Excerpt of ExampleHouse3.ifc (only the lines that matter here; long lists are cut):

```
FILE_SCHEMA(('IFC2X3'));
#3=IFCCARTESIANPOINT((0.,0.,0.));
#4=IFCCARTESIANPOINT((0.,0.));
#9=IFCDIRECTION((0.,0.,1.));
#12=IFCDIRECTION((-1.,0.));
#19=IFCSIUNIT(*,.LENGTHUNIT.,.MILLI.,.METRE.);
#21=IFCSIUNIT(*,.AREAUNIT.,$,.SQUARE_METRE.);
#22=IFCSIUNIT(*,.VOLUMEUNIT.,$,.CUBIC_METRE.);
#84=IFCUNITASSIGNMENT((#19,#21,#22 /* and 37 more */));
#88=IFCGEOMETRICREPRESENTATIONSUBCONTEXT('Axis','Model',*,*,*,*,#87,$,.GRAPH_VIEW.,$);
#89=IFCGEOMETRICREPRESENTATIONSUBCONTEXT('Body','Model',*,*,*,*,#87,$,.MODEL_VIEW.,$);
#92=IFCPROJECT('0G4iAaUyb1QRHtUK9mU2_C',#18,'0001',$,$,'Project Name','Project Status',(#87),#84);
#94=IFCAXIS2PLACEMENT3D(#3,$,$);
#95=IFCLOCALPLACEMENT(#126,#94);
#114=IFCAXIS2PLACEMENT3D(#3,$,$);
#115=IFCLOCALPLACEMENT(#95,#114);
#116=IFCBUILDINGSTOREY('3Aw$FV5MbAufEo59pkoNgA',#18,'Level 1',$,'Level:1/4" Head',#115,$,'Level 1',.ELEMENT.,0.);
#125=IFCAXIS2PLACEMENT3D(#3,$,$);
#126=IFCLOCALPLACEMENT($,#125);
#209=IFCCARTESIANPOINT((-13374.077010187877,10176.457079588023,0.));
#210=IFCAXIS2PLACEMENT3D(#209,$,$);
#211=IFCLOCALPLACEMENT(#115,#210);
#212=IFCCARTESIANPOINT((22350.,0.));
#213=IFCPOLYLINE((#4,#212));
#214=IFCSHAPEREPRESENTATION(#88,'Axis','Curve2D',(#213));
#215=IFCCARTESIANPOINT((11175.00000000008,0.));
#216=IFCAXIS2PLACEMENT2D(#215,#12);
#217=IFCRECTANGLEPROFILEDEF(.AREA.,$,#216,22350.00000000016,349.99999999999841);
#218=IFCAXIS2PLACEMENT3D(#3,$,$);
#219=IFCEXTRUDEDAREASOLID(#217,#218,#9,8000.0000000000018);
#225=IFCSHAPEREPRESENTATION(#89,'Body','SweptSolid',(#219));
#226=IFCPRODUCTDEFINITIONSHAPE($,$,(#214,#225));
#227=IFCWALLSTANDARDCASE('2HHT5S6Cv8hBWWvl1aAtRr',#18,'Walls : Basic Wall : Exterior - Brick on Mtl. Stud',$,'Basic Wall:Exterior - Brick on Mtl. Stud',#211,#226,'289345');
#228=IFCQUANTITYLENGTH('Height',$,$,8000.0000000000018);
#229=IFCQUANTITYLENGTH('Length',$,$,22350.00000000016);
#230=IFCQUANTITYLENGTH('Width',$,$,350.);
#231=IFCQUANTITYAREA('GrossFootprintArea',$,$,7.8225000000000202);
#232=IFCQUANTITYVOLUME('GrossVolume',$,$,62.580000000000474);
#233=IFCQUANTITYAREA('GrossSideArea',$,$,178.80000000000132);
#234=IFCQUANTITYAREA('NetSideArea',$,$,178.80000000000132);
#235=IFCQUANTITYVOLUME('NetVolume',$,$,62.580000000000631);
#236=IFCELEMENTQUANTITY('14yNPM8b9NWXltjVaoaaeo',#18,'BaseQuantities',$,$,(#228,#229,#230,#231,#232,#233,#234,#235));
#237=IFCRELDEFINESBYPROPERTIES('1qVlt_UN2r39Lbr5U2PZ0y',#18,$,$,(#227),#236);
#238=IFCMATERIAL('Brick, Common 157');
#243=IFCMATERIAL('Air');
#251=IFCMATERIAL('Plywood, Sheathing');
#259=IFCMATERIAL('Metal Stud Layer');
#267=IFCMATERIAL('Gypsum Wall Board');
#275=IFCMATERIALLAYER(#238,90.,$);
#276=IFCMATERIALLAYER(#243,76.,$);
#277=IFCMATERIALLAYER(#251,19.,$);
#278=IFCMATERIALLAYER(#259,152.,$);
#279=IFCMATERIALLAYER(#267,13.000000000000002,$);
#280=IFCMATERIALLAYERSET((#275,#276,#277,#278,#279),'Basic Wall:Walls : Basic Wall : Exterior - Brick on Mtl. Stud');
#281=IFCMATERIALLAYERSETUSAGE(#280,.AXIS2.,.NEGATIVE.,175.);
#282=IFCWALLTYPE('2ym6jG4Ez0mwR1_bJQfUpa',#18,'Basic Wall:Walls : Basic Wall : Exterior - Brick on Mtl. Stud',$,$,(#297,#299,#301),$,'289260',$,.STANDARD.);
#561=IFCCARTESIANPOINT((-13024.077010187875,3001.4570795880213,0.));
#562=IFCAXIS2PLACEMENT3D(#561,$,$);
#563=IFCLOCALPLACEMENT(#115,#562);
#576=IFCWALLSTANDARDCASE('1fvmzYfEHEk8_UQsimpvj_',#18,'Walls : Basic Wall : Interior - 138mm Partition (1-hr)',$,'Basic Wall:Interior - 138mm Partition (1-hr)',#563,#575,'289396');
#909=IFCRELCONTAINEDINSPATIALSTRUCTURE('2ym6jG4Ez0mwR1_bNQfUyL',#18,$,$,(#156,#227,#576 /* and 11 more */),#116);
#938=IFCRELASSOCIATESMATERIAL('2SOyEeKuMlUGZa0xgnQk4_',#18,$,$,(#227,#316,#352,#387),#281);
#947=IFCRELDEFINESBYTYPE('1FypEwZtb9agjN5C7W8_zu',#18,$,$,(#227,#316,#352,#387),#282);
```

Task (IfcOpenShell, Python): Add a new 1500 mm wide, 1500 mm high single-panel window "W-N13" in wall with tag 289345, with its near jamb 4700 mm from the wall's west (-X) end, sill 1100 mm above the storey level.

```python
import numpy as np
import ifcopenshell
import ifcopenshell.api.feature
import ifcopenshell.api.geometry
import ifcopenshell.api.pset
import ifcopenshell.api.root
import ifcopenshell.api.spatial
import ifcopenshell.api.type
import ifcopenshell.geom
import ifcopenshell.util.element
import ifcopenshell.util.placement
import ifcopenshell.util.representation
import ifcopenshell.util.shape
import ifcopenshell.util.unit

model = ifcopenshell.open("ExampleHouse3.ifc")
unit_scale = ifcopenshell.util.unit.calculate_unit_scale(model)
area_scale = ifcopenshell.util.unit.calculate_unit_scale(model, "AREAUNIT")
volume_scale = ifcopenshell.util.unit.calculate_unit_scale(model, "VOLUMEUNIT")
settings = ifcopenshell.geom.settings()


def volume(element):
    """Net volume in cubic metres, openings subtracted."""
    shape = ifcopenshell.geom.create_shape(settings, element)
    return ifcopenshell.util.shape.get_volume(shape.geometry)


wall = model.by_guid("2HHT5S6Cv8hBWWvl1aAtRr")
storey = ifcopenshell.util.element.get_container(wall, ifc_class="IfcBuildingStorey")
context = ifcopenshell.util.representation.get_context(model, "Model", "Body", "MODEL_VIEW")
before = volume(wall)

width, height, from_end, sill = 1.5, 1.5, 4.7, 1.1  # metres

# The wall runs along its own X axis, and the end named is its -X end.
wall_shape = ifcopenshell.geom.create_shape(settings, wall)
x, y, z = ifcopenshell.util.shape.get_vertices(wall_shape.geometry).T
start = x.min() + from_end
face, thickness = float(y.min()), float(y.max() - y.min())
wall_matrix = ifcopenshell.util.placement.get_local_placement(wall.ObjectPlacement)
level = ifcopenshell.util.placement.get_local_placement(storey.ObjectPlacement)[2, 3]


def in_wall(x, y):
    """Placement at x, y metres in the wall's axes, at sill height."""
    matrix = wall_matrix.copy()
    matrix[:, 3] = wall_matrix @ np.array([x / unit_scale, y / unit_scale, 0.0, 1.0])
    matrix[2, 3] = level + sill / unit_scale
    return matrix


# Opening: a box that overshoots both wall faces by 50 mm.
opening = ifcopenshell.api.root.create_entity(model, ifc_class="IfcOpeningElement")
box = ifcopenshell.api.geometry.add_wall_representation(
    model, context=context, length=width, height=height, thickness=thickness + 0.1
)
ifcopenshell.api.geometry.assign_representation(model, product=opening, representation=box)
ifcopenshell.api.geometry.edit_object_placement(model, product=opening, matrix=in_wall(start, face - 0.05), is_si=False)
ifcopenshell.api.feature.add_feature(model, feature=opening, element=wall)

window = ifcopenshell.api.root.create_entity(model, ifc_class="IfcWindow", name="W-N13")
window.OverallWidth, window.OverallHeight = width / unit_scale, height / unit_scale
body = ifcopenshell.api.geometry.add_window_representation(
    model,
    context=context,
    overall_width=window.OverallWidth,
    overall_height=window.OverallHeight,
    partition_type="SINGLE_PANEL",
)
ifcopenshell.api.geometry.assign_representation(model, product=window, representation=body)
ifcopenshell.api.spatial.assign_container(model, products=[window], relating_structure=storey)
fills = ifcopenshell.api.feature.add_filling(model, opening=opening, element=window)
fills.OwnerHistory = window.OwnerHistory  # required in IFC2X3

# IFC2X3 keeps the operation on the window style.
style = ifcopenshell.api.root.create_entity(model, ifc_class="IfcWindowStyle", name="W-N13")
style.OperationType, style.ConstructionType = "SINGLE_PANEL", "NOTDEFINED"
style.ParameterTakesPrecedence = style.Sizeable = False
ifcopenshell.api.type.assign_type(model, related_objects=[window], relating_type=style)

# Centre the window in the wall's thickness.
ifcopenshell.api.geometry.edit_object_placement(model, product=window, matrix=in_wall(start, face), is_si=False)
window_shape = ifcopenshell.geom.create_shape(settings, window)
depth = ifcopenshell.util.shape.get_vertices(window_shape.geometry)[:, 1]
offset = face + thickness / 2 - (depth.min() + depth.max()) / 2
ifcopenshell.api.geometry.edit_object_placement(model, product=window, matrix=in_wall(start, offset), is_si=False)

after = volume(wall)

# Update the wall's stored quantities.
qto = model.by_id(ifcopenshell.util.element.get_pset(wall, "BaseQuantities", should_inherit=False)["id"])
ifcopenshell.api.pset.edit_qto(model, qto=qto, properties={
    "NetSideArea": after / thickness / area_scale,
    "NetVolume": after / volume_scale,
})

print(f"wall volume {before:.3f} -> {after:.3f} m3")

model.write("ExampleHouse3_edited.ifc")
```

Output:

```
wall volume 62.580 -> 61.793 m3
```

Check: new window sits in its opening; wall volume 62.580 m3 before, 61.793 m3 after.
